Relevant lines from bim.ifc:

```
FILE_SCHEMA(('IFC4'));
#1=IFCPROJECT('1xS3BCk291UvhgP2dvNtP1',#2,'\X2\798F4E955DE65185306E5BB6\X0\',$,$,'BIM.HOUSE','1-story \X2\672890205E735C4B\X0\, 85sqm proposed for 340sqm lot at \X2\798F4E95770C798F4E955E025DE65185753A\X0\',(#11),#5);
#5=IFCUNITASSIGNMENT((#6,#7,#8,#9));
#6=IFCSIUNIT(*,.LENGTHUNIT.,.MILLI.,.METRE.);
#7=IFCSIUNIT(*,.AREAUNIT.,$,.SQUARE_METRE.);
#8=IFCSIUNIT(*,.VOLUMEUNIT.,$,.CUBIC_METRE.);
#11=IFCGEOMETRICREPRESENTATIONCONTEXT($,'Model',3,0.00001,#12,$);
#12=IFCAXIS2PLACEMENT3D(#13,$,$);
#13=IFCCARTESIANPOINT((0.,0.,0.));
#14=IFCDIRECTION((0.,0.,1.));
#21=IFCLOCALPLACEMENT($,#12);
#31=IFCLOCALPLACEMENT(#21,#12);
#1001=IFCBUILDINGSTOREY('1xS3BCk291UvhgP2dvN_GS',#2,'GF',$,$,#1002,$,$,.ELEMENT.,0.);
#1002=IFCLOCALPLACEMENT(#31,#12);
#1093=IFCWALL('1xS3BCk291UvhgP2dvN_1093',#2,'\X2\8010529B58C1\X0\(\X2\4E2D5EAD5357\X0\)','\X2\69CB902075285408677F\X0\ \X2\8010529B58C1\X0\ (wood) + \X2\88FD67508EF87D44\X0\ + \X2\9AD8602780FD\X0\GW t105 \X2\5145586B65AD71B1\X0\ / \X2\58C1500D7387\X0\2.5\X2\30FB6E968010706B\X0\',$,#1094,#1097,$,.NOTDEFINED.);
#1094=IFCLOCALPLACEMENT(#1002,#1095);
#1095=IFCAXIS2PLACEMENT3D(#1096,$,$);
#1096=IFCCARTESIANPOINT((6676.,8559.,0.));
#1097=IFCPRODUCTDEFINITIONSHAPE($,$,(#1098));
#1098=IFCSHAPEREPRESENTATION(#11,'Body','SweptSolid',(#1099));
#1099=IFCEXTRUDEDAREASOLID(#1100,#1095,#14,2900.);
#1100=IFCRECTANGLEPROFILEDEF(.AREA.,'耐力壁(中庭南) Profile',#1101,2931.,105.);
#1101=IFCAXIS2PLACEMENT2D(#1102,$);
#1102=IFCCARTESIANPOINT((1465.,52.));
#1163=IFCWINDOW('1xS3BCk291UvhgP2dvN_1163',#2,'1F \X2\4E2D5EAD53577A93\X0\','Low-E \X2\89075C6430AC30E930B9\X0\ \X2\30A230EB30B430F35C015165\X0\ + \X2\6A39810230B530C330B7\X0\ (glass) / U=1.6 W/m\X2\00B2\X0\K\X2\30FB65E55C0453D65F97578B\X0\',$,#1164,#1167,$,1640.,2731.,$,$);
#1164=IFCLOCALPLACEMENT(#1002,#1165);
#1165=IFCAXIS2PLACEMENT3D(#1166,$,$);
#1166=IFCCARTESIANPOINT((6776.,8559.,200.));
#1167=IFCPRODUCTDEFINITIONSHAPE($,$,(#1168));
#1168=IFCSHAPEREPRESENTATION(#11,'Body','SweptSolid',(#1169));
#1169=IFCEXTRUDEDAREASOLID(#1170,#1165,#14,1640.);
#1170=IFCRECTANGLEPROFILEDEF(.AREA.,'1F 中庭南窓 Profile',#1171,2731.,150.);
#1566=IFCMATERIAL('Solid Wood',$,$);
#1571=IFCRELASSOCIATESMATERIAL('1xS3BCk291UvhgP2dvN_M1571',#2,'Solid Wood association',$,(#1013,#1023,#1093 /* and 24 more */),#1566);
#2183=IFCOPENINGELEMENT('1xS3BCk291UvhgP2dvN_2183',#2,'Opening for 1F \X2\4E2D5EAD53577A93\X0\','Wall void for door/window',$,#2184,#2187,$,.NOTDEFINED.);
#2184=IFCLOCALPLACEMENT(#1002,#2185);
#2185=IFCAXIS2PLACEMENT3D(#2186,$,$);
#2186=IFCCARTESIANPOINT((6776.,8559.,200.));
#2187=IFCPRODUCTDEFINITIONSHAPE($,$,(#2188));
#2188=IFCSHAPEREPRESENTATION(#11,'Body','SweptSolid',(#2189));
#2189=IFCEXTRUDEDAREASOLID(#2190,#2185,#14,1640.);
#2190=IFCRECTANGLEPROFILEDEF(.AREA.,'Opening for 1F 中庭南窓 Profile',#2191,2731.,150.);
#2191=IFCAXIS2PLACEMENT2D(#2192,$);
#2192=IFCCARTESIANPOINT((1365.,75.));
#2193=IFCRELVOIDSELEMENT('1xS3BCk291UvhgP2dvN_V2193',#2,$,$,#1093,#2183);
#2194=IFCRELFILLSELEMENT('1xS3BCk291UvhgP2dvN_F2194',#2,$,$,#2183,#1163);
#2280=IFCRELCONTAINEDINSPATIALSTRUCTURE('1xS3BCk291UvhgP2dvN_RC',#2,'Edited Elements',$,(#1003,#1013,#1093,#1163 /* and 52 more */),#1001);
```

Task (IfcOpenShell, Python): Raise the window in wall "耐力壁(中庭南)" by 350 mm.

```python
import numpy as np
import ifcopenshell
import ifcopenshell.api.geometry
import ifcopenshell.util.placement
import ifcopenshell.util.unit

model = ifcopenshell.open("bim.ifc")
unit_scale = ifcopenshell.util.unit.calculate_unit_scale(model)

window = model.by_guid("1xS3BCk291UvhgP2dvN_1163")
opening = window.FillsVoids[0].RelatingOpeningElement
dz = 350.0

shift = np.array([0.0, 0.0, dz])
# The window is not placed relative to its opening, so move both.
for product in (opening, window):
    matrix = ifcopenshell.util.placement.get_local_placement(product.ObjectPlacement)
    matrix[:3, 3] += shift
    ifcopenshell.api.geometry.edit_object_placement(model, product=product, matrix=matrix, is_si=False)

print(f"moved by {dz * unit_scale:+.3f} m")

model.write("bim_updated.ifc")
```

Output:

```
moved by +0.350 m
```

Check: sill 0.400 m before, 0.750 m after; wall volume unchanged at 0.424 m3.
